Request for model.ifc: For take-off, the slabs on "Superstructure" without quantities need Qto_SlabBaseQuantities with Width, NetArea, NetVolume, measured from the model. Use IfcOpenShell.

First a look at what the model holds.

```python
import ifcopenshell
import ifcopenshell.util.element
import ifcopenshell.util.unit

model = ifcopenshell.open("model.ifc")
print(model.schema)
for unit_type in ("LENGTHUNIT", "AREAUNIT", "VOLUMEUNIT"):
    print(unit_type, ifcopenshell.util.unit.calculate_unit_scale(model, unit_type))
storey = next(s for s in model.by_type("IfcBuildingStorey") if s.Name == "Superstructure")
slabs = [e for e in ifcopenshell.util.element.get_decomposition(storey) if e.is_a("IfcSlab")]
for e in sorted(slabs, key=lambda e: e.id()):
    print(e.id(), e.is_a(), e.Name, list(ifcopenshell.util.element.get_psets(e, qtos_only=True)), sep=" | ")
```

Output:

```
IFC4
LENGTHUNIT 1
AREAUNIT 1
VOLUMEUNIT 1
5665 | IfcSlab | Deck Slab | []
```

```python
import ifcopenshell
import ifcopenshell.api.pset
import ifcopenshell.geom
import ifcopenshell.util.element
import ifcopenshell.util.shape
import ifcopenshell.util.unit

model = ifcopenshell.open("model.ifc")
unit_scale = ifcopenshell.util.unit.calculate_unit_scale(model)
area_scale = ifcopenshell.util.unit.calculate_unit_scale(model, "AREAUNIT")
volume_scale = ifcopenshell.util.unit.calculate_unit_scale(model, "VOLUMEUNIT")
settings = ifcopenshell.geom.settings()

storey = next(s for s in model.by_type("IfcBuildingStorey") if s.Name == "Superstructure")
slabs = [e for e in ifcopenshell.util.element.get_decomposition(storey) if e.is_a("IfcSlab")]

for e in sorted(slabs, key=lambda e: e.id()):
    if ifcopenshell.util.element.get_psets(e, qtos_only=True, should_inherit=False):
        continue
    # Geometry comes back in metres, in the element's own axes.
    shape = ifcopenshell.geom.create_shape(settings, e)
    values = {
        "Width": ifcopenshell.util.shape.get_z(shape.geometry) / unit_scale,
        "NetArea": ifcopenshell.util.shape.get_footprint_area(shape.geometry) / area_scale,
        "NetVolume": ifcopenshell.util.shape.get_volume(shape.geometry) / volume_scale,
    }
    qto = ifcopenshell.api.pset.add_qto(model, product=e, name="Qto_SlabBaseQuantities")
    ifcopenshell.api.pset.edit_qto(model, qto=qto, properties=values)
    print(e.id(), {k: round(v, 3) for k, v in values.items()})

model.write("model_v2.ifc")
```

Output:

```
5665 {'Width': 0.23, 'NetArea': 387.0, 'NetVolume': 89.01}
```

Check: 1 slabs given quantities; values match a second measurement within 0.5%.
